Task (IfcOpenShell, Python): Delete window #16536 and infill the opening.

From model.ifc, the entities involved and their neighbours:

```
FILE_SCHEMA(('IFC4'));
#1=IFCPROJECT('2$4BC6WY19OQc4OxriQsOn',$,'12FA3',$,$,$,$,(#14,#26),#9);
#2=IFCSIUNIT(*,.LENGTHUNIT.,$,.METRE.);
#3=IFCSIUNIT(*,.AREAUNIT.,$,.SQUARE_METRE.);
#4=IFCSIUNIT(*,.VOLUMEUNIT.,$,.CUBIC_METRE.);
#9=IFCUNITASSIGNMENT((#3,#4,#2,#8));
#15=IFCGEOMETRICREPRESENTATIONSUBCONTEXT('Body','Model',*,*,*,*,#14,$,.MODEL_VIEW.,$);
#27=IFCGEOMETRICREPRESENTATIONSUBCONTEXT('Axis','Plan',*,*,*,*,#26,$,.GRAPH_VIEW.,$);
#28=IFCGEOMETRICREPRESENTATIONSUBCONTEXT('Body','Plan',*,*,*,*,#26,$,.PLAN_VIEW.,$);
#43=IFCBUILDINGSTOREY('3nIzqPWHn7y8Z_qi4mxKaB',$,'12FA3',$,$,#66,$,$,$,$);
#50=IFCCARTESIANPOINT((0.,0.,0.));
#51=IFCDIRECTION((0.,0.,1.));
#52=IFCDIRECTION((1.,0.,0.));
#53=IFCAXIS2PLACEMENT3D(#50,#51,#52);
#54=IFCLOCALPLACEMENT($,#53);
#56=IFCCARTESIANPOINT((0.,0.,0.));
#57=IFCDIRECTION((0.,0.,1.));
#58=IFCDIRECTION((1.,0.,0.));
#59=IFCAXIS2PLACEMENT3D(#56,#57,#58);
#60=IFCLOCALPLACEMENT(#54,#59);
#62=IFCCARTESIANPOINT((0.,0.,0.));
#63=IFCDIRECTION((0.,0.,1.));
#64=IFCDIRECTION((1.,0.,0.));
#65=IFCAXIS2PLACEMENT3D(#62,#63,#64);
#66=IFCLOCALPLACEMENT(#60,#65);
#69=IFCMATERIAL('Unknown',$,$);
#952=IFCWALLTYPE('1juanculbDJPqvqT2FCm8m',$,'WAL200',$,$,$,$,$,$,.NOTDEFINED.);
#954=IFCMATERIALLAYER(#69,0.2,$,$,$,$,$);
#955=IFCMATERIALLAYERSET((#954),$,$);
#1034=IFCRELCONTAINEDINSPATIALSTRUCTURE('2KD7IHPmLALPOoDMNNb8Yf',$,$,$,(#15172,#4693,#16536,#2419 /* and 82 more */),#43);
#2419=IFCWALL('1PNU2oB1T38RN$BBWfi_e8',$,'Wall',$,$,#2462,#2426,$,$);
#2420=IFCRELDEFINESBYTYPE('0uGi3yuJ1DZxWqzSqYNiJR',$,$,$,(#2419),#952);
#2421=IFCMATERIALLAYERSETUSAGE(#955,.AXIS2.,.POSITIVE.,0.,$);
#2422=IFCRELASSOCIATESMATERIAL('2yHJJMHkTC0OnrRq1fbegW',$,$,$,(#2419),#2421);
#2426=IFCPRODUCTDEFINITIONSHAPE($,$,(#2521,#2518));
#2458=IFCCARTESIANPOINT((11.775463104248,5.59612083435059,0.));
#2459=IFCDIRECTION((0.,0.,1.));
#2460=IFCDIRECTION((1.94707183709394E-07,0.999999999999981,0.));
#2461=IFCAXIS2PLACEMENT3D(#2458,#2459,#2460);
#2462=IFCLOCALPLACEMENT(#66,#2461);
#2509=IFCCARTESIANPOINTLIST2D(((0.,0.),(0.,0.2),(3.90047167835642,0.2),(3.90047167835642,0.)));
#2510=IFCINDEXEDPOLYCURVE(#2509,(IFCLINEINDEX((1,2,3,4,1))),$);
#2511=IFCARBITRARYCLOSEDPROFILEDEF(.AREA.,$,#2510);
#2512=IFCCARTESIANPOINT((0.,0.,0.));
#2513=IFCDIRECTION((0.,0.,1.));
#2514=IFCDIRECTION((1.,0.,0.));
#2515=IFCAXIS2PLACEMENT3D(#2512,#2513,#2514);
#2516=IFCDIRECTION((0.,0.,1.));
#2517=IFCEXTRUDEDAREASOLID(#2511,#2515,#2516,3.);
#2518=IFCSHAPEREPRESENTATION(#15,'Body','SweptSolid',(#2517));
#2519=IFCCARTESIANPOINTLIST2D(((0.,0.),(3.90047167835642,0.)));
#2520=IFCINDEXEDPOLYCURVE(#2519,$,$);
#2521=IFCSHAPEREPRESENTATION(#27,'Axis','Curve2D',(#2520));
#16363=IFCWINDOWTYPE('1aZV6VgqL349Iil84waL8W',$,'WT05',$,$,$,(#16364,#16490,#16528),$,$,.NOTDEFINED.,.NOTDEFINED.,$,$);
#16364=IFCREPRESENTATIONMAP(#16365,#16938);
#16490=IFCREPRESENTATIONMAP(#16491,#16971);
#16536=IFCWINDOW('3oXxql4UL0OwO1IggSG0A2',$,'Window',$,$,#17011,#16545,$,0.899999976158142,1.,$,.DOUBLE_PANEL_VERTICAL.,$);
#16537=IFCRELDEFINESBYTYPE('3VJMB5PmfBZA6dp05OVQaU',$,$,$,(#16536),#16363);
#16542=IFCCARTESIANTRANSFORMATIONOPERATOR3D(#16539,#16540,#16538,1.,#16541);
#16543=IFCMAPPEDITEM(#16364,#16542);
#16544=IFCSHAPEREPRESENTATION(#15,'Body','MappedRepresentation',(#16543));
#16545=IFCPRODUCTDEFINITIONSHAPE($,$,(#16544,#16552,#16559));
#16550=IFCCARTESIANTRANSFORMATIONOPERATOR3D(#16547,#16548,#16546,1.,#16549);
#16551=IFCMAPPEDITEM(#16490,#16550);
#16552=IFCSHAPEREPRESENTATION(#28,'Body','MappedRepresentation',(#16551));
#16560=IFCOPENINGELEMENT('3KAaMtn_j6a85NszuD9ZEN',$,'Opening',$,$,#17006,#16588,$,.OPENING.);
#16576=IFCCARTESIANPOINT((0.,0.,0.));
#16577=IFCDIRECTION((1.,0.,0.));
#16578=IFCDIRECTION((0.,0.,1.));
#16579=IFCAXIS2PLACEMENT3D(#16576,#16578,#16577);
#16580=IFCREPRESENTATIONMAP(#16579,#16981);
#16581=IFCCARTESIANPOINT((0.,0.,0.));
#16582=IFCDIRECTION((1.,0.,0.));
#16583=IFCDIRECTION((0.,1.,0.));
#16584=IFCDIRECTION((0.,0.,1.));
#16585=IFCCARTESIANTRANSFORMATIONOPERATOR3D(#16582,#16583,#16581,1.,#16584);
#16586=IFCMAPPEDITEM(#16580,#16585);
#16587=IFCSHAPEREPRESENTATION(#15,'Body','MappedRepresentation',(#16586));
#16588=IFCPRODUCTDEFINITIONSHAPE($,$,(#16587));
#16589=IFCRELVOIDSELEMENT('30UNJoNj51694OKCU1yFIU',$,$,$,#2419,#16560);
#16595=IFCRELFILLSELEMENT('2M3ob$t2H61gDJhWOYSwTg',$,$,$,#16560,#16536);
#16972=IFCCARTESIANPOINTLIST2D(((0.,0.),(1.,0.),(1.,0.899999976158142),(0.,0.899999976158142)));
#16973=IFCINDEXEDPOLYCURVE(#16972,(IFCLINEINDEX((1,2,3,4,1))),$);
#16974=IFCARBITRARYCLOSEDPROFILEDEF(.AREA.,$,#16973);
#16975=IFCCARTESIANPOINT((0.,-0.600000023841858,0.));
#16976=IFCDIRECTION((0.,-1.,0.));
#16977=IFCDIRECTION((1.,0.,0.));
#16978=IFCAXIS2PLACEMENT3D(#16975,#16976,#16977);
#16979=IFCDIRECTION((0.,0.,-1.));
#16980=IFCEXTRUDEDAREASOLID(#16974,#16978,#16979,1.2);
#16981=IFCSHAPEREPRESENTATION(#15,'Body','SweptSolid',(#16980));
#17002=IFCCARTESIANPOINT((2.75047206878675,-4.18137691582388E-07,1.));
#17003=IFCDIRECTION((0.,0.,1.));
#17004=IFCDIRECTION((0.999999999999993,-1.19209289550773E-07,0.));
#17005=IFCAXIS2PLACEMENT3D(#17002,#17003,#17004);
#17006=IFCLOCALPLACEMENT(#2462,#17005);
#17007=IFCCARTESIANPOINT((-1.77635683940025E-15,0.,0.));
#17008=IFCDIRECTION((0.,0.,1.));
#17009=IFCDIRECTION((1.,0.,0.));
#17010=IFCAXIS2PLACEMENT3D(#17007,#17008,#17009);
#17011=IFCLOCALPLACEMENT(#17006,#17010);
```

```python
import ifcopenshell
import ifcopenshell.api.feature
import ifcopenshell.api.root
import ifcopenshell.geom
import ifcopenshell.util.shape

model = ifcopenshell.open("model.ifc")
settings = ifcopenshell.geom.settings()


def volume(element):
    """Net volume in cubic metres, openings subtracted."""
    shape = ifcopenshell.geom.create_shape(settings, element)
    return ifcopenshell.util.shape.get_volume(shape.geometry)


window = model.by_guid("3oXxql4UL0OwO1IggSG0A2")
opening = window.FillsVoids[0].RelatingOpeningElement
wall = opening.VoidsElements[0].RelatingBuildingElement
before = volume(wall)

ifcopenshell.api.root.remove_product(model, product=window)
ifcopenshell.api.feature.remove_feature(model, feature=opening)

after = volume(wall)

print(f"wall volume {before:.3f} -> {after:.3f} m3")

model.write("model_edited.ifc")
```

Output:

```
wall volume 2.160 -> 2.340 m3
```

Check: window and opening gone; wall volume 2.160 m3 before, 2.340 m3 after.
